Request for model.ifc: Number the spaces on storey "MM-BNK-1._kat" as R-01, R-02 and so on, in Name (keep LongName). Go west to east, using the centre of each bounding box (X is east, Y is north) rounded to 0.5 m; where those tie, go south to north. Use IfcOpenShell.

First a look at what the model holds.

```python
import ifcopenshell
import ifcopenshell.util.element
import ifcopenshell.util.placement

model = ifcopenshell.open("model.ifc")
print(model.schema)
storey = next(s for s in model.by_type("IfcBuildingStorey") if s.Name == "MM-BNK-1._kat")
spaces = [e for e in ifcopenshell.util.element.get_decomposition(storey) if e.is_a("IfcSpace")]
for e in sorted(spaces, key=lambda e: e.id()):
    origin = ifcopenshell.util.placement.get_local_placement(e.ObjectPlacement)[:3, 3]
    print(e.id(), e.Name, e.LongName, origin.round(2) + 0.0, sep=" | ")
```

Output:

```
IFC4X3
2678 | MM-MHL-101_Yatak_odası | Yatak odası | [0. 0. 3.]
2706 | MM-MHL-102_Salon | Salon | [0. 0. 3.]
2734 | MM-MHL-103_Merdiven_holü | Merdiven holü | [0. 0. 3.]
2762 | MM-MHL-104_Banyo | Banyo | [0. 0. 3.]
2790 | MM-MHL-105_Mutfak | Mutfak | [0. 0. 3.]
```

```python
import ifcopenshell
import ifcopenshell.geom
import ifcopenshell.util.element
import ifcopenshell.util.shape

model = ifcopenshell.open("model.ifc")
settings = ifcopenshell.geom.settings()
settings.set("use-world-coords", True)


def centre(element):
    shape = ifcopenshell.geom.create_shape(settings, element)
    return ifcopenshell.util.shape.get_bbox_centroid(shape.geometry)


storey = next(s for s in model.by_type("IfcBuildingStorey") if s.Name == "MM-BNK-1._kat")
spaces = [e for e in ifcopenshell.util.element.get_decomposition(storey) if e.is_a("IfcSpace")]

# Insertion points can sit at a corner or the storey origin, so sort by the geometry (in metres).
centres = {e: centre(e) for e in spaces}
spaces.sort(key=lambda e: (round(centres[e][0] / 0.5), centres[e][1]))

for i, e in enumerate(spaces, start=1):
    number = f"R-{i:02d}"
    e.Name = number
    print(e.id(), number)

model.write("model_updated.ifc")
```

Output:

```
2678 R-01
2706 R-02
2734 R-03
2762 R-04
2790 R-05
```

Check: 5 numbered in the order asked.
